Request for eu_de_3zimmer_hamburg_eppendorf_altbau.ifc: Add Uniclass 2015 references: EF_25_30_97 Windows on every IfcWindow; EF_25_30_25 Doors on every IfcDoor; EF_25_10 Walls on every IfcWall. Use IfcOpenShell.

First a look at what the model holds.

```python
import ifcopenshell

model = ifcopenshell.open("eu_de_3zimmer_hamburg_eppendorf_altbau.ifc")
print(model.schema)
print("classifications:", [c.Name for c in model.by_type("IfcClassification")])
for ifc_class in ("IfcDoor", "IfcRoof", "IfcStair", "IfcWall", "IfcWindow"):
    print(ifc_class, len(model.by_type(ifc_class)))
```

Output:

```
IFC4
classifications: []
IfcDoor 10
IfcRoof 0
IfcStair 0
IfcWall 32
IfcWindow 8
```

```python
import ifcopenshell
import ifcopenshell.api.classification

model = ifcopenshell.open("eu_de_3zimmer_hamburg_eppendorf_altbau.ifc")

system = ifcopenshell.api.classification.add_classification(model, classification="Uniclass 2015")

codes = {
    "IfcWindow": ("EF_25_30_97", "Windows"),
    "IfcDoor": ("EF_25_30_25", "Doors"),
    "IfcWall": ("EF_25_10", "Walls"),
}
for ifc_class, (code, name) in codes.items():
    products = model.by_type(ifc_class)
    ifcopenshell.api.classification.add_reference(
        model, products=products, classification=system, identification=code, name=name
    )
    print(code, len(products))

model.write("eu_de_3zimmer_hamburg_eppendorf_altbau_updated.ifc")
```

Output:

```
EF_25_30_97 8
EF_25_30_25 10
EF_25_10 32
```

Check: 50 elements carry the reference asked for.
